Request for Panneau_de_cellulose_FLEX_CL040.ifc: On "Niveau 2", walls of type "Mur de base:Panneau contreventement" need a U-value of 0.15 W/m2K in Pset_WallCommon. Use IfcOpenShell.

First a look at what the model holds.

```python
import ifcopenshell
import ifcopenshell.util.element

model = ifcopenshell.open("Panneau_de_cellulose_FLEX_CL040.ifc")
print(model.schema)
storey = next(s for s in model.by_type("IfcBuildingStorey") if s.Name == "Niveau 2")
walls = [e for e in ifcopenshell.util.element.get_decomposition(storey) if e.is_a("IfcWall")]
seen = {}
for e in walls:
    element_type = ifcopenshell.util.element.get_type(e)
    key = (element_type.Name if element_type != e and element_type else None, ifcopenshell.util.element.get_pset(e, "Pset_WallCommon", "ThermalTransmittance"))
    seen[key] = seen.get(key, 0) + 1
for (name, value), count in sorted(seen.items(), key=str):
    print(count, "x", name, "|", value)
```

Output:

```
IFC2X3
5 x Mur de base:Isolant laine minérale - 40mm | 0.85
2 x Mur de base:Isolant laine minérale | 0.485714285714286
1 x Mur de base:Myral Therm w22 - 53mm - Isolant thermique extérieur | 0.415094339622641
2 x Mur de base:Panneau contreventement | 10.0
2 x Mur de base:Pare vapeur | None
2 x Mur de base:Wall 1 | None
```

```python
import ifcopenshell
import ifcopenshell.api.pset
import ifcopenshell.util.element

model = ifcopenshell.open("Panneau_de_cellulose_FLEX_CL040.ifc")

storey = next(s for s in model.by_type("IfcBuildingStorey") if s.Name == "Niveau 2")
walls = [e for e in ifcopenshell.util.element.get_decomposition(storey) if e.is_a("IfcWall")]

count = 0
for e in walls:
    element_type = ifcopenshell.util.element.get_type(e)
    if element_type in (None, e) or element_type.Name != "Mur de base:Panneau contreventement":
        continue
    # add_pset returns the element's existing set when there is one.
    pset = ifcopenshell.api.pset.add_pset(model, product=e, name="Pset_WallCommon")
    ifcopenshell.api.pset.edit_pset(model, pset=pset, properties={"ThermalTransmittance": 0.15})
    count += 1

print(count, "walls updated")

model.write("Panneau_de_cellulose_FLEX_CL040-out.ifc")
```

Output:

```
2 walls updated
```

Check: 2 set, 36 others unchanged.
